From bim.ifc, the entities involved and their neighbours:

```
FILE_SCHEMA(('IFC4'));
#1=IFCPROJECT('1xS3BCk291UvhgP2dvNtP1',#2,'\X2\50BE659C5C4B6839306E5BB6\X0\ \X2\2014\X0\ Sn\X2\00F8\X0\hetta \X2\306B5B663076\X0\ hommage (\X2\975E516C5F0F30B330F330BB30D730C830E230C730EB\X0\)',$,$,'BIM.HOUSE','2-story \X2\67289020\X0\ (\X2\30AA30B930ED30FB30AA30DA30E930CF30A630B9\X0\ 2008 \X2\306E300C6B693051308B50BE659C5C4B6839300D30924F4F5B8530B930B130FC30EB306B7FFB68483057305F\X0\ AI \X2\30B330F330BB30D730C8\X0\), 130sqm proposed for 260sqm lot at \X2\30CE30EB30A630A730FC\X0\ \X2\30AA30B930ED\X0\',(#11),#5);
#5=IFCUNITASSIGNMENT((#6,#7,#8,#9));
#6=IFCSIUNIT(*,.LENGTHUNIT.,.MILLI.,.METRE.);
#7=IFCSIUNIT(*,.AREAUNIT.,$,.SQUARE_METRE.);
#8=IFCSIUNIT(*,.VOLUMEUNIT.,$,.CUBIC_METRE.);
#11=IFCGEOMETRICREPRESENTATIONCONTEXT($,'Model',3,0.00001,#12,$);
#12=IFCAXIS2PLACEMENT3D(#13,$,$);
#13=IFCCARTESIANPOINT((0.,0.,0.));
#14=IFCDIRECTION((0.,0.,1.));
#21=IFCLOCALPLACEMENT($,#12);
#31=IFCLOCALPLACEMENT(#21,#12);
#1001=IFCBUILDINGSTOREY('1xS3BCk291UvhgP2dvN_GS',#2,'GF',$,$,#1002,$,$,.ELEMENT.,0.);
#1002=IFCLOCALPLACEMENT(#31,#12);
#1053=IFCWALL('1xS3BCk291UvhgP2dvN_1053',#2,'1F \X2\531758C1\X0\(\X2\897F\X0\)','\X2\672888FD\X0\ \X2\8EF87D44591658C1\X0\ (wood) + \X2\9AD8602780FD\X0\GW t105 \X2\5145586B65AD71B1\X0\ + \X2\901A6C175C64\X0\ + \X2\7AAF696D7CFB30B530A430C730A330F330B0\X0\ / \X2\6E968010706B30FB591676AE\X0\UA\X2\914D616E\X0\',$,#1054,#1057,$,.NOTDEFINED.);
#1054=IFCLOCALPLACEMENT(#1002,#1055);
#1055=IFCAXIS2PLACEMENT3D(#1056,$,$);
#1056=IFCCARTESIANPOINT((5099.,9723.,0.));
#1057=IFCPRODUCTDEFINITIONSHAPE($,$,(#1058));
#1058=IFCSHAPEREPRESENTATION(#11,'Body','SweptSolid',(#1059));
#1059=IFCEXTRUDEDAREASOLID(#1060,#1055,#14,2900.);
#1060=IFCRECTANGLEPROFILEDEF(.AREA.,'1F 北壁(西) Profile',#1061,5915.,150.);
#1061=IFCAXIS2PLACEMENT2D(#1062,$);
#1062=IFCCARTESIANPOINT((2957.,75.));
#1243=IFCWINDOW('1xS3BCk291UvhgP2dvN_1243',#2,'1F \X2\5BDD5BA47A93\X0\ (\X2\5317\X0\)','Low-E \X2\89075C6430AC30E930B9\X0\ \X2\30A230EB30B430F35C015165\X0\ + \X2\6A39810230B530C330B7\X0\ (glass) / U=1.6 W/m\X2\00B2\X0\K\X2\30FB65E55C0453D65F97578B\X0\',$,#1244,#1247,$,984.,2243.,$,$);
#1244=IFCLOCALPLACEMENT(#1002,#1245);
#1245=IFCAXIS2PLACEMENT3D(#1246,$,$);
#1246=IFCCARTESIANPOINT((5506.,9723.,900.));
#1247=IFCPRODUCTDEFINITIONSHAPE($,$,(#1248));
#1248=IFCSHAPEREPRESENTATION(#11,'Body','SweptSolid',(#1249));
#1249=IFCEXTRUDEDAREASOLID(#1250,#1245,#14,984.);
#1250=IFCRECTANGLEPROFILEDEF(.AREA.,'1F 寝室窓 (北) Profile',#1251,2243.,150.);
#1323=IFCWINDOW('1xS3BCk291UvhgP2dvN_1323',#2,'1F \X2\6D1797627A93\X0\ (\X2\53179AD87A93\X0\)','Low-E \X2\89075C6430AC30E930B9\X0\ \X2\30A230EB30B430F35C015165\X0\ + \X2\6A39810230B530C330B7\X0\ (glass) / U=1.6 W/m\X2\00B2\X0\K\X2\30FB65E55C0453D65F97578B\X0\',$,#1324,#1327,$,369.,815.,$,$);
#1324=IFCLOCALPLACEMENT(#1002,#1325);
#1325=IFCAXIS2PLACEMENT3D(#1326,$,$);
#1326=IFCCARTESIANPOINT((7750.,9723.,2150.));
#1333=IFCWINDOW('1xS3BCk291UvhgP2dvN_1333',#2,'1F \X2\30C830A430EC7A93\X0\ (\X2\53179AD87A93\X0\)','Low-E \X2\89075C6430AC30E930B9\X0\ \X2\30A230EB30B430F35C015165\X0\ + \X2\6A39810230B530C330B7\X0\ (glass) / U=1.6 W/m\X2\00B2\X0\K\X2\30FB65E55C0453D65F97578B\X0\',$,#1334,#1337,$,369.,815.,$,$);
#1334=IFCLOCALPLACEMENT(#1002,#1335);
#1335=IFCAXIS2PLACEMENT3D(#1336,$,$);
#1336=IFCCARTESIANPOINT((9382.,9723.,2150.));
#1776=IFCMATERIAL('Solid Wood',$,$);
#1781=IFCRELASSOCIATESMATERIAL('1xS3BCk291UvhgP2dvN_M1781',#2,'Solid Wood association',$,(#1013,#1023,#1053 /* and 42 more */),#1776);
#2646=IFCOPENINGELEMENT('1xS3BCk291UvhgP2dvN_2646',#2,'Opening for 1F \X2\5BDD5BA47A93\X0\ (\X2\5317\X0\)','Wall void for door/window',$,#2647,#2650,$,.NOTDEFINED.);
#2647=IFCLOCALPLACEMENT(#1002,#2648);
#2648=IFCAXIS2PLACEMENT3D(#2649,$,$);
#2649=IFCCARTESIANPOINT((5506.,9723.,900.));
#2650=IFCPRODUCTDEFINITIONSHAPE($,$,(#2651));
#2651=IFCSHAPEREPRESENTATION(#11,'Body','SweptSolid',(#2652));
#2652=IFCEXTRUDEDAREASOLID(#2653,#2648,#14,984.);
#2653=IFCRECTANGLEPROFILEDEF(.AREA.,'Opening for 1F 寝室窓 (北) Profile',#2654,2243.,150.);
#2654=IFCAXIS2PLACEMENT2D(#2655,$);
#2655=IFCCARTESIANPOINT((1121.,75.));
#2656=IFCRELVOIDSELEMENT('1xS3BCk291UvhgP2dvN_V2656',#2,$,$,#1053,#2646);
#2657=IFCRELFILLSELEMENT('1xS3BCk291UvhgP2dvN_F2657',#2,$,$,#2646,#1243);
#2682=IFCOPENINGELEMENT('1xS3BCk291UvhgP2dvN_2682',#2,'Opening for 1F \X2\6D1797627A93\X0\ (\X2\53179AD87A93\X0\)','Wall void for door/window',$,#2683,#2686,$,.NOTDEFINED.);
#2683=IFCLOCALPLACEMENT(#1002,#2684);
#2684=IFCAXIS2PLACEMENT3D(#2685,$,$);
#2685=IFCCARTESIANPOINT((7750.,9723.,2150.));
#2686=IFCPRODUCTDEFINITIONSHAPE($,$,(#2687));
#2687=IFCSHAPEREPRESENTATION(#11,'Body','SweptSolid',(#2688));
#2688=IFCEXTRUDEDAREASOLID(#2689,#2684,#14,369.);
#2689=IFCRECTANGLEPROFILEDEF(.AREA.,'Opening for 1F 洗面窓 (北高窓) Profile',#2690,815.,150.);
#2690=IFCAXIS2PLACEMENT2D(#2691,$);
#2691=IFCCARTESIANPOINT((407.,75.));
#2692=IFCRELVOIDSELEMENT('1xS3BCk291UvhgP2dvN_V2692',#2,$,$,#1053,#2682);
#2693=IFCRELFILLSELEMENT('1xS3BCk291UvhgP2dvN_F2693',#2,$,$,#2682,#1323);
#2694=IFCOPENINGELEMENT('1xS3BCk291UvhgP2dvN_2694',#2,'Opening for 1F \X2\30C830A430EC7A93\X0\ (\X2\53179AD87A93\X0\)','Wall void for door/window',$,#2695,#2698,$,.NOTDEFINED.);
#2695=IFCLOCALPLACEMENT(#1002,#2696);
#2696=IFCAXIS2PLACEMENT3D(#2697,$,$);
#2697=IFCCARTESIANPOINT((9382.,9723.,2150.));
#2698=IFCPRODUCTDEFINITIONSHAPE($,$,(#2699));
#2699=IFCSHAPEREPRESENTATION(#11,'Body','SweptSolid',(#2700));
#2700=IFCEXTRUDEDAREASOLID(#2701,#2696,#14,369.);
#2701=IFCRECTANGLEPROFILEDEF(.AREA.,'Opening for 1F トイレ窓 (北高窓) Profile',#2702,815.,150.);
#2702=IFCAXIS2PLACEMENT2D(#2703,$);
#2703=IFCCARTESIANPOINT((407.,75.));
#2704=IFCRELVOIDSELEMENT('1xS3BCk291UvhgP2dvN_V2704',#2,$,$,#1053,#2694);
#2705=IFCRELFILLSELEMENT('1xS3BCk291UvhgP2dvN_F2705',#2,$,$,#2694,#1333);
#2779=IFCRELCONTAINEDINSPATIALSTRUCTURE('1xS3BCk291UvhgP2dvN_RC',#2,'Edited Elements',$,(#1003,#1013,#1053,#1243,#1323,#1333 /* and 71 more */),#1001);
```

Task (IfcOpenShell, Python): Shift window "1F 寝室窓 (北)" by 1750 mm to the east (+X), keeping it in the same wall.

```python
import ifcopenshell
import ifcopenshell.api.geometry
import ifcopenshell.util.placement

model = ifcopenshell.open("bim.ifc")

window = model.by_guid("1xS3BCk291UvhgP2dvN_1243")
opening = window.FillsVoids[0].RelatingOpeningElement
wall = opening.VoidsElements[0].RelatingBuildingElement

wall_matrix = ifcopenshell.util.placement.get_local_placement(wall.ObjectPlacement)
shift = wall_matrix[:3, 0] * 1750.0
before = ifcopenshell.util.placement.get_local_placement(window.ObjectPlacement)[:3, 3].copy()

# The window is not placed relative to its opening, so move both.
for product in (opening, window):
    matrix = ifcopenshell.util.placement.get_local_placement(product.ObjectPlacement)
    matrix[:3, 3] += shift
    ifcopenshell.api.geometry.edit_object_placement(model, product=product, matrix=matrix, is_si=False)

after = ifcopenshell.util.placement.get_local_placement(window.ObjectPlacement)[:3, 3]
print("window moved by", (after - before).round(3) + 0.0)

model.write("bim-out.ifc")
```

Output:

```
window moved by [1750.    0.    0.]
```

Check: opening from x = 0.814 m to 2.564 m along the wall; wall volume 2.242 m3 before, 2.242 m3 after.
